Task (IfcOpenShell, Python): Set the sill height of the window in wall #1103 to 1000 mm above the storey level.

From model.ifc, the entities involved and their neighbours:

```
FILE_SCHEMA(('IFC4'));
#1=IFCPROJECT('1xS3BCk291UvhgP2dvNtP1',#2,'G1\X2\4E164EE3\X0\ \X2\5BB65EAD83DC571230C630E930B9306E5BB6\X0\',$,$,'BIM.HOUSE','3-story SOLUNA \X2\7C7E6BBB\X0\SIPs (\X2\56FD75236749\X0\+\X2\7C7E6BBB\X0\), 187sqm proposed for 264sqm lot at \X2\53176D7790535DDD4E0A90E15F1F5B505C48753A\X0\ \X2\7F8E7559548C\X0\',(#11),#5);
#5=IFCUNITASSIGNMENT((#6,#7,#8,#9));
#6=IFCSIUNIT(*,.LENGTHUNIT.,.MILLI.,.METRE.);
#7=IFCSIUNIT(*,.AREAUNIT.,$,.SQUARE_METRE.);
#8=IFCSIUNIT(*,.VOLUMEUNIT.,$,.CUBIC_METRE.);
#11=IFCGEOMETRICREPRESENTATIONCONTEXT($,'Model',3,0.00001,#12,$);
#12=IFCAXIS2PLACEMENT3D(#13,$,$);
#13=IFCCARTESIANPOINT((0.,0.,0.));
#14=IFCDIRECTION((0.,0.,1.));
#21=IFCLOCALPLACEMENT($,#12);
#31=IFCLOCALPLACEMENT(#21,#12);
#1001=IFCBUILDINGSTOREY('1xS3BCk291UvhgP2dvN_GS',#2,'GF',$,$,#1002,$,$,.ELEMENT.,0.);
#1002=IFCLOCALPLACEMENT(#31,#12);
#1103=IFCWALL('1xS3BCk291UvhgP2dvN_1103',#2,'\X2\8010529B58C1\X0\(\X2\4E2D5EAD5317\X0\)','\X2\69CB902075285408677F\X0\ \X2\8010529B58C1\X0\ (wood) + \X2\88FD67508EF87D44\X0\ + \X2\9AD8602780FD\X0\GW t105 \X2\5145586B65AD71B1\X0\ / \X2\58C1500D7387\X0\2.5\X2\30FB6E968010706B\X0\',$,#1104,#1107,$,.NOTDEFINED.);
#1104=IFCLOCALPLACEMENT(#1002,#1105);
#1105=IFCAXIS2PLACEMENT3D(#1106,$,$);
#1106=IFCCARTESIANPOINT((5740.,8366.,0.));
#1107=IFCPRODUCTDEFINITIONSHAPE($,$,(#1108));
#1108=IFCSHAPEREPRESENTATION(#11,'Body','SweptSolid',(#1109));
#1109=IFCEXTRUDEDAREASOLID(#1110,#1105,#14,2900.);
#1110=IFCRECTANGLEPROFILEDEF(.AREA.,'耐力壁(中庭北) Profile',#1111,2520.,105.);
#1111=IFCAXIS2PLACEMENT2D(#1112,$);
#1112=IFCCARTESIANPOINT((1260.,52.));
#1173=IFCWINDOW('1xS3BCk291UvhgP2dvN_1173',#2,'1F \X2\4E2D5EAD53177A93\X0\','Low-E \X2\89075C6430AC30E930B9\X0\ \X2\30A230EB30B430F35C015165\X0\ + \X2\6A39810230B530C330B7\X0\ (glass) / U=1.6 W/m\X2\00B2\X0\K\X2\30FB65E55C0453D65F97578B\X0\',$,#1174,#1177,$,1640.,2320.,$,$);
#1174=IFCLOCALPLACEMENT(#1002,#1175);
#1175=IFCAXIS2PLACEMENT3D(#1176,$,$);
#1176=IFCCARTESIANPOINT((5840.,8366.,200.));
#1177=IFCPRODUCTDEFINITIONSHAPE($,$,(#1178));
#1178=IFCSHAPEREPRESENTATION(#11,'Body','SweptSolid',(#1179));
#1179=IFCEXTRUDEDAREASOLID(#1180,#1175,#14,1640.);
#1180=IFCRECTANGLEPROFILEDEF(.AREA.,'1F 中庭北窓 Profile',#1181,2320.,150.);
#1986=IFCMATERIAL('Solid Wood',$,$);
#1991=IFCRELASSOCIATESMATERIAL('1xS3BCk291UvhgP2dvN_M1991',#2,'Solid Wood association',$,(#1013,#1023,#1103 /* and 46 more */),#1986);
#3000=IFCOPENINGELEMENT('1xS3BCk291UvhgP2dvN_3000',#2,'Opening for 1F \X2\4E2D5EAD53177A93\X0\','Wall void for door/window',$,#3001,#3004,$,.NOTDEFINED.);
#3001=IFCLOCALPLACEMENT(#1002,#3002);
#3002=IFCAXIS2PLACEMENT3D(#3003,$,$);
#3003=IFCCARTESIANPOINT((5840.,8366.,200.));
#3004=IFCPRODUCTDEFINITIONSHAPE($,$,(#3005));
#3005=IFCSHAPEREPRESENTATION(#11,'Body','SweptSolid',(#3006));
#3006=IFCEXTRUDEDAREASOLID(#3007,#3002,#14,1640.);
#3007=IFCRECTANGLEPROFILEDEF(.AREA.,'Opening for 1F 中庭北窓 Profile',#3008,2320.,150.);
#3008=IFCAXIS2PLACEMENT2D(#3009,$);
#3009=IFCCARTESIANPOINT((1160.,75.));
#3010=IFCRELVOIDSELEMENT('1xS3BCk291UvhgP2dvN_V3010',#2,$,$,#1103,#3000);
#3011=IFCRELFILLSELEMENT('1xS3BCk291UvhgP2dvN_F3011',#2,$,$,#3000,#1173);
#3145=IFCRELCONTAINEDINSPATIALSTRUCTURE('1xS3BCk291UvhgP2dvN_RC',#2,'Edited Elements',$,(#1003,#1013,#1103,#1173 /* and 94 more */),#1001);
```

```python
import numpy as np
import ifcopenshell
import ifcopenshell.api.geometry
import ifcopenshell.geom
import ifcopenshell.util.element
import ifcopenshell.util.placement
import ifcopenshell.util.shape
import ifcopenshell.util.unit

model = ifcopenshell.open("model.ifc")
unit_scale = ifcopenshell.util.unit.calculate_unit_scale(model)

window = model.by_guid("1xS3BCk291UvhgP2dvN_1173")
opening = window.FillsVoids[0].RelatingOpeningElement
storey = ifcopenshell.util.element.get_container(window, ifc_class="IfcBuildingStorey")
level = ifcopenshell.util.placement.get_local_placement(storey.ObjectPlacement)[2, 3]

# The opening's origin need not be at the sill, so measure its lowest point.
shape = ifcopenshell.geom.create_shape(ifcopenshell.geom.settings(), opening)
bottom = ifcopenshell.util.shape.get_shape_bottom_elevation(shape, shape.geometry) / unit_scale
dz = level + 1 / unit_scale - bottom

shift = np.array([0.0, 0.0, dz])
# The window is not placed relative to its opening, so move both.
for product in (opening, window):
    matrix = ifcopenshell.util.placement.get_local_placement(product.ObjectPlacement)
    matrix[:3, 3] += shift
    ifcopenshell.api.geometry.edit_object_placement(model, product=product, matrix=matrix, is_si=False)

print(f"moved by {dz * unit_scale:+.3f} m")

model.write("model_rev.ifc")
```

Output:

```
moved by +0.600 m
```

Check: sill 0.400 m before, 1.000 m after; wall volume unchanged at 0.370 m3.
